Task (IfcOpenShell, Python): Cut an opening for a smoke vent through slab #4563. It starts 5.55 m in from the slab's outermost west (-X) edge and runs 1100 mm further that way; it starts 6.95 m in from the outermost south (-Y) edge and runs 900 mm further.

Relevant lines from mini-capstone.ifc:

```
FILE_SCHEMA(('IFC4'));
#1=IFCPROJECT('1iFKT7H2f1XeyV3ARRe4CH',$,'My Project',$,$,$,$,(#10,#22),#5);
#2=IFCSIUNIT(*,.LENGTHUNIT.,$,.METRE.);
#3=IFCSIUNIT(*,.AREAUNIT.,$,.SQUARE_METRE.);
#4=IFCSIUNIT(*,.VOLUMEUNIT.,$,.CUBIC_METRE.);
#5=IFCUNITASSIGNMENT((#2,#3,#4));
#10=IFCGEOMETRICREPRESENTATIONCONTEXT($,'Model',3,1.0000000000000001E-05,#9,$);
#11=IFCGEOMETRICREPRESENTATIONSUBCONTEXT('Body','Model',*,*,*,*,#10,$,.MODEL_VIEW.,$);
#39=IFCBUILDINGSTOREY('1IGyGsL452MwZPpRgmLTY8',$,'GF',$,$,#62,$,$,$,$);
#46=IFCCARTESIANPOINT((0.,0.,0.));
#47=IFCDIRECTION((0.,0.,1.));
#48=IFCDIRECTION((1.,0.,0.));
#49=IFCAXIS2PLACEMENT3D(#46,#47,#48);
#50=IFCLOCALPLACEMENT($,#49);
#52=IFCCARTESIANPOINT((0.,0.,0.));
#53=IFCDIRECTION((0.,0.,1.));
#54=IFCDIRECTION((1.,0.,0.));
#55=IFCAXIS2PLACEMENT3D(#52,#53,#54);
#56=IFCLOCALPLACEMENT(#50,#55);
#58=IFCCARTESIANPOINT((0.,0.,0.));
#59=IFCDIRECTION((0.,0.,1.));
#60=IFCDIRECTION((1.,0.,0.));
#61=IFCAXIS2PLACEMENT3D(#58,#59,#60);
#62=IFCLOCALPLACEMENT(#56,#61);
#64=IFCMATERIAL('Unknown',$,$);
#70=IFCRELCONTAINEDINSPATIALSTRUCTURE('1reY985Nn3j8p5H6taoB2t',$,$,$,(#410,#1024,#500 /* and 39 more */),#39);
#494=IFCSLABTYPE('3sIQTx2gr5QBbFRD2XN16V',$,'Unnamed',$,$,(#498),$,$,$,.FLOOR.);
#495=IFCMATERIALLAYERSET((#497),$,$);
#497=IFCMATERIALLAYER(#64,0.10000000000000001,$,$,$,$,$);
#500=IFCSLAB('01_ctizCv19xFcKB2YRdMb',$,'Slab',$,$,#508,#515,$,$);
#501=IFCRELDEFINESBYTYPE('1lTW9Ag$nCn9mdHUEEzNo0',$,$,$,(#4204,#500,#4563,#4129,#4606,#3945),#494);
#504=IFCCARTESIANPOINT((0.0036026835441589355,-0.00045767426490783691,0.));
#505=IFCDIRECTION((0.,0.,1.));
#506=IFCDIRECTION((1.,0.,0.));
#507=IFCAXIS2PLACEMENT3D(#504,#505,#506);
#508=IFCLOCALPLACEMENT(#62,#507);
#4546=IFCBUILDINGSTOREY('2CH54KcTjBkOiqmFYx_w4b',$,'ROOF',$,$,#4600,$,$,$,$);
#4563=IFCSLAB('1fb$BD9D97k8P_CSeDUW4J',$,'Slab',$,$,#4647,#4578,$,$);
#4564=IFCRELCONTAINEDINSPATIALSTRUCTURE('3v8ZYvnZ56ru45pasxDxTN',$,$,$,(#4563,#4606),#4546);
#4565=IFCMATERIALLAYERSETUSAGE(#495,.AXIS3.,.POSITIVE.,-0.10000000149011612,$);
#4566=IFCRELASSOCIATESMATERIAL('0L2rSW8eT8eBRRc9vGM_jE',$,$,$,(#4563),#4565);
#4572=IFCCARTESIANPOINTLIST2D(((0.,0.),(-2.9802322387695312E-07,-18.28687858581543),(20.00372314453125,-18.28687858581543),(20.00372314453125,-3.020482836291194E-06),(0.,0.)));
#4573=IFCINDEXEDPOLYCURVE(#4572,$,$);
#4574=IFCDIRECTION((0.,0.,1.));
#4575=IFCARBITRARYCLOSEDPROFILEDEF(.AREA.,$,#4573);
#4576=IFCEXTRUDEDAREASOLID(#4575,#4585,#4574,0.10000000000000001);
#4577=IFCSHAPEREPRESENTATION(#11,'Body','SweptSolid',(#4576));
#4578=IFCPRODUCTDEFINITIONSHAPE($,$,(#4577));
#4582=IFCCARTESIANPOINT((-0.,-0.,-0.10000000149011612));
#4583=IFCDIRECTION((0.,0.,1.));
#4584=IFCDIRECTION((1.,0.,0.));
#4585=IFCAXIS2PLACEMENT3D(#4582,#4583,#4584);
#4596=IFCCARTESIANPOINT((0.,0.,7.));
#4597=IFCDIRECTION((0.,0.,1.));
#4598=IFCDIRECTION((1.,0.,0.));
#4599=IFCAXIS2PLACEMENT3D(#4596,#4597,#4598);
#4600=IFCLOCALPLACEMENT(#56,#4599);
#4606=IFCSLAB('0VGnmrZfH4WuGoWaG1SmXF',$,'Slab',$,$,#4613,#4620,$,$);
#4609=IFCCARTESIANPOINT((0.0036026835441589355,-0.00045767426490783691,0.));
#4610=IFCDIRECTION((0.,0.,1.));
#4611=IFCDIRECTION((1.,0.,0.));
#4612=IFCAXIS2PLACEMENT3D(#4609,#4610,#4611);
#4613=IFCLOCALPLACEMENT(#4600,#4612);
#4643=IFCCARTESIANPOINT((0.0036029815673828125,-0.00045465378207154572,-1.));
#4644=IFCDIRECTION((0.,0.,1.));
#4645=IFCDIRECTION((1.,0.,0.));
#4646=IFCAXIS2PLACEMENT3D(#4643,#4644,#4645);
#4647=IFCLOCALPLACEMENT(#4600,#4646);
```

```python
import numpy as np
import ifcopenshell
import ifcopenshell.api.feature
import ifcopenshell.api.geometry
import ifcopenshell.api.root
import ifcopenshell.geom
import ifcopenshell.util.placement
import ifcopenshell.util.representation
import ifcopenshell.util.shape
import ifcopenshell.util.unit

model = ifcopenshell.open("mini-capstone.ifc")
unit_scale = ifcopenshell.util.unit.calculate_unit_scale(model)
settings = ifcopenshell.geom.settings()


def volume(element):
    """Net volume in cubic metres, openings subtracted."""
    shape = ifcopenshell.geom.create_shape(settings, element)
    return ifcopenshell.util.shape.get_volume(shape.geometry)


slab = model.by_guid("1fb$BD9D97k8P_CSeDUW4J")
before = volume(slab)

# Extent in the slab's own axes, in metres. The edges named are its -X and -Y sides.
slab_shape = ifcopenshell.geom.create_shape(settings, slab)
vertices = ifcopenshell.util.shape.get_vertices(slab_shape.geometry)
x_min, y_min, bottom = vertices.min(axis=0)
top = vertices[:, 2].max()

opening = ifcopenshell.api.root.create_entity(model, ifc_class="IfcOpeningElement", name="Smoke vent opening", predefined_type="OPENING")
context = ifcopenshell.util.representation.get_context(model, "Model", "Body", "MODEL_VIEW")
width, depth = 1.1, 0.9
outline = [(0.0, 0.0), (width, 0.0), (width, depth), (0.0, depth), (0.0, 0.0)]
# Overshoot both faces by 50 mm so the cut is clean.
shape = ifcopenshell.api.geometry.add_slab_representation(
    model, context=context, depth=top - bottom + 0.1, polyline=outline
)
ifcopenshell.api.geometry.assign_representation(model, product=opening, representation=shape)

matrix = ifcopenshell.util.placement.get_local_placement(slab.ObjectPlacement)
matrix[:, 3] = matrix @ np.append(np.array([x_min + 5.55, y_min + 6.95, bottom - 0.05]) / unit_scale, 1.0)
ifcopenshell.api.geometry.edit_object_placement(model, product=opening, matrix=matrix, is_si=False)
ifcopenshell.api.feature.add_feature(model, feature=opening, element=slab)

after = volume(slab)

print(f"slab volume {before:.3f} -> {after:.3f} m3")

model.write("mini-capstone_updated.ifc")
```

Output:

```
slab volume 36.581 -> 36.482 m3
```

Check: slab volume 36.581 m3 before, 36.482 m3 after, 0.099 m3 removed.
